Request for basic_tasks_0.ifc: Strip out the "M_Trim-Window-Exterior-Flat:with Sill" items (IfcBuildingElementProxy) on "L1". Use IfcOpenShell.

First a look at what the model holds.

```python
import ifcopenshell
import ifcopenshell.util.element

model = ifcopenshell.open("basic_tasks_0.ifc")
print(model.schema)
storey = next(s for s in model.by_type("IfcBuildingStorey") if s.Name == "L1")
proxies = [e for e in ifcopenshell.util.element.get_decomposition(storey) if e.is_a("IfcBuildingElementProxy")]
seen = {}
for e in proxies:
    element_type = ifcopenshell.util.element.get_type(e)
    name = element_type.Name if element_type not in (None, e) else None
    seen[name] = seen.get(name, 0) + 1
for name, count in sorted(seen.items(), key=str):
    print(count, "x", name)
```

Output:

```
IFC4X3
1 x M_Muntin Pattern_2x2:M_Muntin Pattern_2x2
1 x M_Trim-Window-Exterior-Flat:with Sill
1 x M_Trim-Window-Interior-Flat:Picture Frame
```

```python
import ifcopenshell
import ifcopenshell.api.root
import ifcopenshell.util.element

model = ifcopenshell.open("basic_tasks_0.ifc")

storey = next(s for s in model.by_type("IfcBuildingStorey") if s.Name == "L1")
proxies = [e for e in ifcopenshell.util.element.get_decomposition(storey) if e.is_a("IfcBuildingElementProxy")]
targets = [e for e in proxies if (t := ifcopenshell.util.element.get_type(e)) not in (None, e) and t.Name == "M_Trim-Window-Exterior-Flat:with Sill"]

for e in targets:
    ifcopenshell.api.root.remove_product(model, product=e)
print(len(targets), "removed")

model.write("basic_tasks_0_v2.ifc")
```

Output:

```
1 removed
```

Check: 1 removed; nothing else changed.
